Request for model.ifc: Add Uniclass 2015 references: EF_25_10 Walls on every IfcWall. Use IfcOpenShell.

First a look at what the model holds.

```python
import ifcopenshell

model = ifcopenshell.open("model.ifc")
print(model.schema)
print("classifications:", [c.Name for c in model.by_type("IfcClassification")])
for ifc_class in ("IfcDoor", "IfcRoof", "IfcStair", "IfcWall", "IfcWindow"):
    print(ifc_class, len(model.by_type(ifc_class)))
```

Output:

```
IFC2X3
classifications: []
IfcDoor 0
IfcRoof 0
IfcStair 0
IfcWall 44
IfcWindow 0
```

```python
import ifcopenshell
import ifcopenshell.api.classification

model = ifcopenshell.open("model.ifc")

# IFC2X3 requires Source and Edition and has no link from the project to the system.
system = model.create_entity("IfcClassification", Source="NBS", Edition="2015", Name="Uniclass 2015")

codes = {
    "IfcWall": ("EF_25_10", "Walls"),
}
for ifc_class, (code, name) in codes.items():
    products = model.by_type(ifc_class)
    ifcopenshell.api.classification.add_reference(
        model, products=products, classification=system, identification=code, name=name
    )
    print(code, len(products))

model.write("model_rev.ifc")
```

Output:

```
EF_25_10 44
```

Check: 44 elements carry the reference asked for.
